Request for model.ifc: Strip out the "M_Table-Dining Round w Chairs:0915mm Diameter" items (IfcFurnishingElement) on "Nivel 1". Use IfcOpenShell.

First a look at what the model holds.

```python
import ifcopenshell
import ifcopenshell.util.element

model = ifcopenshell.open("model.ifc")
print(model.schema)
storey = next(s for s in model.by_type("IfcBuildingStorey") if s.Name == "Nivel 1")
furniture = [e for e in ifcopenshell.util.element.get_decomposition(storey) if e.is_a("IfcFurnishingElement")]
seen = {}
for e in furniture:
    element_type = ifcopenshell.util.element.get_type(e)
    name = element_type.Name if element_type not in (None, e) else None
    seen[name] = seen.get(name, 0) + 1
for name, count in sorted(seen.items(), key=str):
    print(count, "x", name)
```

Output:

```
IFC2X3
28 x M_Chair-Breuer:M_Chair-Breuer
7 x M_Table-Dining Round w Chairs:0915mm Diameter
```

```python
import ifcopenshell
import ifcopenshell.api.root
import ifcopenshell.util.element

model = ifcopenshell.open("model.ifc")

storey = next(s for s in model.by_type("IfcBuildingStorey") if s.Name == "Nivel 1")
furniture = [e for e in ifcopenshell.util.element.get_decomposition(storey) if e.is_a("IfcFurnishingElement")]
targets = [e for e in furniture if (t := ifcopenshell.util.element.get_type(e)) not in (None, e) and t.Name == "M_Table-Dining Round w Chairs:0915mm Diameter"]

for e in targets:
    ifcopenshell.api.root.remove_product(model, product=e)
print(len(targets), "removed")

model.write("model-out.ifc")
```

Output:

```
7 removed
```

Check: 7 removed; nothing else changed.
